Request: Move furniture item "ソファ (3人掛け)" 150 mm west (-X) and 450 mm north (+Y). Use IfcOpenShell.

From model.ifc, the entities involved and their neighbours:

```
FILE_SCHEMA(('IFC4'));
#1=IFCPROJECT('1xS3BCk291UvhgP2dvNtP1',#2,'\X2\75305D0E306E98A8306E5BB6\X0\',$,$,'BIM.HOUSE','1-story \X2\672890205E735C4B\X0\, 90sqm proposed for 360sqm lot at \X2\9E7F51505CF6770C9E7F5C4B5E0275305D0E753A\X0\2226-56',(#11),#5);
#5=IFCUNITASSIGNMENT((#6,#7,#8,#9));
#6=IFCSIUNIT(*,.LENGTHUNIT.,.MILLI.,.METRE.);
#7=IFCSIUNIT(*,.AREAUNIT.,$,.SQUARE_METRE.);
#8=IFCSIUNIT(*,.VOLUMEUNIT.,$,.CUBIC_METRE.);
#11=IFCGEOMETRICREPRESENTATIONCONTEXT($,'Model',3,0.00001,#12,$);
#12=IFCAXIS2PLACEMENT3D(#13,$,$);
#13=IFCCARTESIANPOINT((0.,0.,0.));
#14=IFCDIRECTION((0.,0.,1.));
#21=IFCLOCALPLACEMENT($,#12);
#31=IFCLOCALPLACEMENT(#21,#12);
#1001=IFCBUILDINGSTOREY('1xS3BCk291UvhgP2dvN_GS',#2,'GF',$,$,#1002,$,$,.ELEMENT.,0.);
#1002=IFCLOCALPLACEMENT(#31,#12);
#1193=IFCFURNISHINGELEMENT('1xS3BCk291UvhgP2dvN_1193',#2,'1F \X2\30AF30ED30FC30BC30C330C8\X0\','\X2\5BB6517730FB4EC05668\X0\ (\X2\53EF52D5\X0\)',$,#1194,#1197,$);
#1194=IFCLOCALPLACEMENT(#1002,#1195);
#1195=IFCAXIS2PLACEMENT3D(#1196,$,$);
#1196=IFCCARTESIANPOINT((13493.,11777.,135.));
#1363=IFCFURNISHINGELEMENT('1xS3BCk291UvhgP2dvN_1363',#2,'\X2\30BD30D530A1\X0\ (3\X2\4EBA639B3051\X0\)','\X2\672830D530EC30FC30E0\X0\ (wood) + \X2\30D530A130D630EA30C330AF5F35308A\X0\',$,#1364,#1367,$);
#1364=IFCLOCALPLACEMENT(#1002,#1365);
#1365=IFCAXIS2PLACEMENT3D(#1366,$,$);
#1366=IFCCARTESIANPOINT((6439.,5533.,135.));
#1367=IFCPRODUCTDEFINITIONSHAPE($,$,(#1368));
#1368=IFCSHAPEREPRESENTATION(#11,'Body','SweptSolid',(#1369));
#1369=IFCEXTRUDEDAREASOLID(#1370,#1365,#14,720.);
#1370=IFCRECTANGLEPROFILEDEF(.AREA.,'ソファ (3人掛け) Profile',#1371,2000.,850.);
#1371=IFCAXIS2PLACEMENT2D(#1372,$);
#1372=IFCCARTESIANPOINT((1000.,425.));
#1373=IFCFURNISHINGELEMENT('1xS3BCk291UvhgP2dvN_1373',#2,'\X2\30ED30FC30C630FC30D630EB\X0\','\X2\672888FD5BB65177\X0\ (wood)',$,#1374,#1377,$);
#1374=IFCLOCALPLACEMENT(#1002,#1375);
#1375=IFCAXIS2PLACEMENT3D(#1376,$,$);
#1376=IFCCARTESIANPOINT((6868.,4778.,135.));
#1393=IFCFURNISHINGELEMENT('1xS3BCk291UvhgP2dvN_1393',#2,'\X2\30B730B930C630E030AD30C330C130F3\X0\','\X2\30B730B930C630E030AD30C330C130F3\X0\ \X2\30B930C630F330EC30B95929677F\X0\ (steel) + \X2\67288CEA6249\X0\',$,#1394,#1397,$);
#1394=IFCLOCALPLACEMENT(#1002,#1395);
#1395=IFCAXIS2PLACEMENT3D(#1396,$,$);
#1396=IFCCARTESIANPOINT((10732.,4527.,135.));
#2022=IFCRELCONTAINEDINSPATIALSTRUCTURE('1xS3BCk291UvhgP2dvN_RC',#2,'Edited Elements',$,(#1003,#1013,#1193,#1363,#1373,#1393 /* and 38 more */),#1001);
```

```python
import ifcopenshell
import ifcopenshell.api.geometry
import ifcopenshell.util.placement

model = ifcopenshell.open("model.ifc")

item = model.by_guid("1xS3BCk291UvhgP2dvN_1363")
matrix = ifcopenshell.util.placement.get_local_placement(item.ObjectPlacement)
matrix[0, 3] -= 150.0
matrix[1, 3] += 450.0
ifcopenshell.api.geometry.edit_object_placement(model, product=item, matrix=matrix, is_si=False)

print(ifcopenshell.util.placement.get_local_placement(item.ObjectPlacement).round(3) + 0.0)

model.write("model_updated.ifc")
```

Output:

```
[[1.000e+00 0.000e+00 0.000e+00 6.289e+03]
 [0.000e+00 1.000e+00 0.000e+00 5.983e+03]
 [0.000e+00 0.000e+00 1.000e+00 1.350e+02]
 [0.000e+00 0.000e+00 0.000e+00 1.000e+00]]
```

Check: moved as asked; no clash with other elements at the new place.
